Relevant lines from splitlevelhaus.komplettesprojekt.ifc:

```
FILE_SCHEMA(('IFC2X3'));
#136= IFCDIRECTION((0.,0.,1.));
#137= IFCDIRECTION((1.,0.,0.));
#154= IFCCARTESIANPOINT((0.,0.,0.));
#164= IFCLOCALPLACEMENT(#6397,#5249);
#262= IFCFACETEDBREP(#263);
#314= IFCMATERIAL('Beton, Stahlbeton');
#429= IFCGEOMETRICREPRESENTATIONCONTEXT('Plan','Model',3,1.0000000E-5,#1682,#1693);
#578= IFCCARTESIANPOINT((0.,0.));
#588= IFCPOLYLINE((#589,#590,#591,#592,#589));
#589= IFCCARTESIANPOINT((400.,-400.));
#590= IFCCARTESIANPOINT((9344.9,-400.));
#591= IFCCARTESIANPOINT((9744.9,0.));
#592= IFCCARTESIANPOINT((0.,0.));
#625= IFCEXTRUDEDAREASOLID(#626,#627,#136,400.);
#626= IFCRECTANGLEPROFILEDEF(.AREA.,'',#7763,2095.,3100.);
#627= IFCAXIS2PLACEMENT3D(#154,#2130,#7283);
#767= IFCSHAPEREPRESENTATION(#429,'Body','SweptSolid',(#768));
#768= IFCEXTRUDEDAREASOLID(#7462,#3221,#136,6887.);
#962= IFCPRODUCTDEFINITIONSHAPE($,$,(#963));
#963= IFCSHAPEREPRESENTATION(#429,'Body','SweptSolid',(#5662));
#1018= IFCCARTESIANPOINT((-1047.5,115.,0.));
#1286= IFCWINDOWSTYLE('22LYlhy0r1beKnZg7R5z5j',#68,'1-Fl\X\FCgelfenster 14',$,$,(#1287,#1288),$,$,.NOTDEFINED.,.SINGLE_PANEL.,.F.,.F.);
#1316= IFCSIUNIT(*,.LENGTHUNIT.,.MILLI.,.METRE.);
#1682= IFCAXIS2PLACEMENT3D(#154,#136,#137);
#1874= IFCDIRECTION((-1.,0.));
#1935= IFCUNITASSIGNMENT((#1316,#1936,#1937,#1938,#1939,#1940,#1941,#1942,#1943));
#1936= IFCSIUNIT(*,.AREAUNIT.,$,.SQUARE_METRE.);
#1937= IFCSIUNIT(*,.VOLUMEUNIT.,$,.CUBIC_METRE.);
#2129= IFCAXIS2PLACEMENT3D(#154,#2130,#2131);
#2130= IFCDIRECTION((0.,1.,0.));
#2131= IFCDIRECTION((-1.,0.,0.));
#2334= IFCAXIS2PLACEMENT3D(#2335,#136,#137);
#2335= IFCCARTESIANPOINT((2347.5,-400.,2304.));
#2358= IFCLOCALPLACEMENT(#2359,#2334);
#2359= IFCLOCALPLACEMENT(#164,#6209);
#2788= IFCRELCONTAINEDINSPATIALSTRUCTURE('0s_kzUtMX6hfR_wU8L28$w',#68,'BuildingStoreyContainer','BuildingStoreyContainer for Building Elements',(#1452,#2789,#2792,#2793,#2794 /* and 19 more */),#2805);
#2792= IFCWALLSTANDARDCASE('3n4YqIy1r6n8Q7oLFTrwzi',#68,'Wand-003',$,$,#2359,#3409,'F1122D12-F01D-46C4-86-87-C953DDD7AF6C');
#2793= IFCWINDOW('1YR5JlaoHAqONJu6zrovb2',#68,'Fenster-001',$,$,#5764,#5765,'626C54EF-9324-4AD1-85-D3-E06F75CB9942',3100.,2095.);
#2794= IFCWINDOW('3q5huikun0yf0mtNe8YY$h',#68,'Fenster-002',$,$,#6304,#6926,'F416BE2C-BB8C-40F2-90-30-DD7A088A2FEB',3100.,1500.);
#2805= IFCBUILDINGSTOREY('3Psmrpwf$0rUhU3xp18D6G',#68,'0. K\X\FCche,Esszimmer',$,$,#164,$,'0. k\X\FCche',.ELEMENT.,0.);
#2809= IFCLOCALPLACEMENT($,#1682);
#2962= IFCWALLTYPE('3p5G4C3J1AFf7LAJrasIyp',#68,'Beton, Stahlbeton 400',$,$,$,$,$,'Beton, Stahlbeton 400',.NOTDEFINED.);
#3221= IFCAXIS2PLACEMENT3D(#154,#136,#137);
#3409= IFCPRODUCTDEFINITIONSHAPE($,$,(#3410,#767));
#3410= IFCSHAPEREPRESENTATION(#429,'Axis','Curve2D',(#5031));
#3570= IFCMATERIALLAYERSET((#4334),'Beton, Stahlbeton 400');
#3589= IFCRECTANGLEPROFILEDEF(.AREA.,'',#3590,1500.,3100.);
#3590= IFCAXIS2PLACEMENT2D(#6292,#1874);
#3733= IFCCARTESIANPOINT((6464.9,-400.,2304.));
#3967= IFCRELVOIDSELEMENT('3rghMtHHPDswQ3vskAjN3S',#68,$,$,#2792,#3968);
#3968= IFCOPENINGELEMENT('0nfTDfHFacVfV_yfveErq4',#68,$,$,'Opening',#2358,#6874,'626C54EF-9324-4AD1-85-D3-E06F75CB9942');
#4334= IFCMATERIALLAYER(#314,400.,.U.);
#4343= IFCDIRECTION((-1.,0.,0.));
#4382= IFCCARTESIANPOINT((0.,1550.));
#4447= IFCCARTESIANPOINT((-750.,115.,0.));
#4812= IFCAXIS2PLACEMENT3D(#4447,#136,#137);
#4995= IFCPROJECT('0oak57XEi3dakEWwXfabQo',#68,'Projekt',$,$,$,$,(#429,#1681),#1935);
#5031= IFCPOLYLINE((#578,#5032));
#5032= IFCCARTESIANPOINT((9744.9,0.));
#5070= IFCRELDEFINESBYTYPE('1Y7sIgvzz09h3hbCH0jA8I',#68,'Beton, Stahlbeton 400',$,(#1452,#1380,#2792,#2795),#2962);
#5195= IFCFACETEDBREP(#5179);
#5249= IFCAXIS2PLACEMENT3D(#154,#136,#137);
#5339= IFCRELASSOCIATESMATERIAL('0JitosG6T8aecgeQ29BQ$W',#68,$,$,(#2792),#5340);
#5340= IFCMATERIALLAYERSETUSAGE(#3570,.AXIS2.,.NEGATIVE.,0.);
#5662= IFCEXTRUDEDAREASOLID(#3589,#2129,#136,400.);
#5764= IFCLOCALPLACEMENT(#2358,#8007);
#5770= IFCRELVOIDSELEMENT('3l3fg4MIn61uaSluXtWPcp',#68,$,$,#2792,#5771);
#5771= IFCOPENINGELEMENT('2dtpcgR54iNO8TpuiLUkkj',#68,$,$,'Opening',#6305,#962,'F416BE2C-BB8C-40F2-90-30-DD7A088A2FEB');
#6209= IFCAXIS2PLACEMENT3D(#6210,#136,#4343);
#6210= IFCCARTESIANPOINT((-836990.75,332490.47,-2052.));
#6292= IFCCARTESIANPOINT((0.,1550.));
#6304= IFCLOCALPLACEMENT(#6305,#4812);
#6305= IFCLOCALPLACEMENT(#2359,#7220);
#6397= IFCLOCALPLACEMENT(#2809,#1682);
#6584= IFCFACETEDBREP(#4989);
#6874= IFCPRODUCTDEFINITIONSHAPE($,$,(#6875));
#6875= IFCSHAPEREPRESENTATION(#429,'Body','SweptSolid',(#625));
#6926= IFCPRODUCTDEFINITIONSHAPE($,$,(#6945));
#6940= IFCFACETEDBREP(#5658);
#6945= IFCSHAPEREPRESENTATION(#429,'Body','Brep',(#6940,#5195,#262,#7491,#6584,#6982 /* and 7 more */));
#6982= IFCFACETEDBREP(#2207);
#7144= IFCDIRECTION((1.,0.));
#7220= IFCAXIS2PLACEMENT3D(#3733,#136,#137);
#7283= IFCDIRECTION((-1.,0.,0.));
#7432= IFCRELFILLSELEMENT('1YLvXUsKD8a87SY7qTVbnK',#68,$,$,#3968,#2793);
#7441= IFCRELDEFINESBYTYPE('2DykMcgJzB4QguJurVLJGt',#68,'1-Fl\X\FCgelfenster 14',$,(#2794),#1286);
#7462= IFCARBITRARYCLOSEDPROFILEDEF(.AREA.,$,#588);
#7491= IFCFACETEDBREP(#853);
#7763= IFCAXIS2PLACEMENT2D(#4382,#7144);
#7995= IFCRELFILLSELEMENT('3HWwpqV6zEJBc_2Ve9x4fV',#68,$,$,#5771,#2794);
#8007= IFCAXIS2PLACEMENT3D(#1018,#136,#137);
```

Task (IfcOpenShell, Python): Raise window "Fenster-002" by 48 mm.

```python
import numpy as np
import ifcopenshell
import ifcopenshell.api.geometry
import ifcopenshell.util.placement
import ifcopenshell.util.unit

model = ifcopenshell.open("splitlevelhaus.komplettesprojekt.ifc")
unit_scale = ifcopenshell.util.unit.calculate_unit_scale(model)

window = model.by_guid("3q5huikun0yf0mtNe8YY$h")
opening = window.FillsVoids[0].RelatingOpeningElement
dz = 0.048 / unit_scale

shift = np.array([0.0, 0.0, dz])
# The window is placed relative to its opening, so it follows when the opening moves.
matrix = ifcopenshell.util.placement.get_local_placement(opening.ObjectPlacement)
matrix[:3, 3] += shift
ifcopenshell.api.geometry.edit_object_placement(
    model, product=opening, matrix=matrix, is_si=False, should_transform_children=True
)

print(f"moved by {dz * unit_scale:+.3f} m")

model.write("splitlevelhaus.komplettesprojekt_updated.ifc")
```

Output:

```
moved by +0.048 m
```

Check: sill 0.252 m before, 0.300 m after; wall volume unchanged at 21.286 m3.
